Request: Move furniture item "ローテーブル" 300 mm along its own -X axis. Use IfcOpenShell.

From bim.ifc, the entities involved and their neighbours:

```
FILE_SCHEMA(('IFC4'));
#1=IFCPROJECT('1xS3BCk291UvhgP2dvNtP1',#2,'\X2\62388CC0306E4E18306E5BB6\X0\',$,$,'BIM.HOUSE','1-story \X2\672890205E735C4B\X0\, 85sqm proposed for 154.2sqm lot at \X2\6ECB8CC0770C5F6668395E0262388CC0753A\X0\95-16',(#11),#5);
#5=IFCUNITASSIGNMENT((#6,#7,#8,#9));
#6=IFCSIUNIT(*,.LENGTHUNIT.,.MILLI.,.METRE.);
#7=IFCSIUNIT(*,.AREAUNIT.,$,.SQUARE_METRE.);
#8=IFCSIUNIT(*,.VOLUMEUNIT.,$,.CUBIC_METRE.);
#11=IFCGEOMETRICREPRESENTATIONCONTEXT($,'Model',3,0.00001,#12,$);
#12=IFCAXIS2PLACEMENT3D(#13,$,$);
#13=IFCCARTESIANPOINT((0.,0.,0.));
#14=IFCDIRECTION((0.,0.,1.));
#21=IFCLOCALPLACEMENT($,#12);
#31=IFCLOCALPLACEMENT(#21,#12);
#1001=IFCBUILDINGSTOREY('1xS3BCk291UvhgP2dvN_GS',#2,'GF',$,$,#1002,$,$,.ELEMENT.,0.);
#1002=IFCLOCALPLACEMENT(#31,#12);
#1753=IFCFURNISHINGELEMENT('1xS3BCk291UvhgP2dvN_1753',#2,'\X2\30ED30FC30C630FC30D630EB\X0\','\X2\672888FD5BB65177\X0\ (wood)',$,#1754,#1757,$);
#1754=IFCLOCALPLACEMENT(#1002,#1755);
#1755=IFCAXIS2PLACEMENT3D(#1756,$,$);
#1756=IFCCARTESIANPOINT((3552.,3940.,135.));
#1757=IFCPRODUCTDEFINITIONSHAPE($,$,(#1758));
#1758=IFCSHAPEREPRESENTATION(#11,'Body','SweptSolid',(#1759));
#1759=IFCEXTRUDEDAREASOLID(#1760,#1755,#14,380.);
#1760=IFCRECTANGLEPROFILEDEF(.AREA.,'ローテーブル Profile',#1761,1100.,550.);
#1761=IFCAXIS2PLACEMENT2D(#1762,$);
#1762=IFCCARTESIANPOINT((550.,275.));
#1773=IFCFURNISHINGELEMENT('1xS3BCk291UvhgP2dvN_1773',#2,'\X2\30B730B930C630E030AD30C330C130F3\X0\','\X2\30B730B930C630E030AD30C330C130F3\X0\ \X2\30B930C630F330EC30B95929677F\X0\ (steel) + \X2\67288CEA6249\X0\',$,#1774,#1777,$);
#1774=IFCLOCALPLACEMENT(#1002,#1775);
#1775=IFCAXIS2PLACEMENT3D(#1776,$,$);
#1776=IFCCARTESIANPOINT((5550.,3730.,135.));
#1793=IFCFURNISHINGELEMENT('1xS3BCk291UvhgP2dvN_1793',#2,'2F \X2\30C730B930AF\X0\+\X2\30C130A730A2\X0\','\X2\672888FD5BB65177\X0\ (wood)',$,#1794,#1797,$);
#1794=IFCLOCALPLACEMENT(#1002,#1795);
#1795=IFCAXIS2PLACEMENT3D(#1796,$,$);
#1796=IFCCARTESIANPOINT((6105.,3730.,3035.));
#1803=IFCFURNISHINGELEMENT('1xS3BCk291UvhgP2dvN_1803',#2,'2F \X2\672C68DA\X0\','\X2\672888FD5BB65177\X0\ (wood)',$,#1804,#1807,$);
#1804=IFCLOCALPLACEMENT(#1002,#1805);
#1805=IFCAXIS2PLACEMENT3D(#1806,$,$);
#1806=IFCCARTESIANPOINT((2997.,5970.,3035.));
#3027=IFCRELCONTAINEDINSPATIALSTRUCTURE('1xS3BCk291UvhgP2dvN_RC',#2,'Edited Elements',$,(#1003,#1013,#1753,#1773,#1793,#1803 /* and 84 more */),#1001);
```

```python
import ifcopenshell
import ifcopenshell.api.geometry
import ifcopenshell.util.placement

model = ifcopenshell.open("bim.ifc")

item = model.by_guid("1xS3BCk291UvhgP2dvN_1753")
matrix = ifcopenshell.util.placement.get_local_placement(item.ObjectPlacement)
matrix[:3, 3] -= matrix[:3, 0] * 300.0
ifcopenshell.api.geometry.edit_object_placement(model, product=item, matrix=matrix, is_si=False)

print(ifcopenshell.util.placement.get_local_placement(item.ObjectPlacement).round(3) + 0.0)

model.write("bim_edited.ifc")
```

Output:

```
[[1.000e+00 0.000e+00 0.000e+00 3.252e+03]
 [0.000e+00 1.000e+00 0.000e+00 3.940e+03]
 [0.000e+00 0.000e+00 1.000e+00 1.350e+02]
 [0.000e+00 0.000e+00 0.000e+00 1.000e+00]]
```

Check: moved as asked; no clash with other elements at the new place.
